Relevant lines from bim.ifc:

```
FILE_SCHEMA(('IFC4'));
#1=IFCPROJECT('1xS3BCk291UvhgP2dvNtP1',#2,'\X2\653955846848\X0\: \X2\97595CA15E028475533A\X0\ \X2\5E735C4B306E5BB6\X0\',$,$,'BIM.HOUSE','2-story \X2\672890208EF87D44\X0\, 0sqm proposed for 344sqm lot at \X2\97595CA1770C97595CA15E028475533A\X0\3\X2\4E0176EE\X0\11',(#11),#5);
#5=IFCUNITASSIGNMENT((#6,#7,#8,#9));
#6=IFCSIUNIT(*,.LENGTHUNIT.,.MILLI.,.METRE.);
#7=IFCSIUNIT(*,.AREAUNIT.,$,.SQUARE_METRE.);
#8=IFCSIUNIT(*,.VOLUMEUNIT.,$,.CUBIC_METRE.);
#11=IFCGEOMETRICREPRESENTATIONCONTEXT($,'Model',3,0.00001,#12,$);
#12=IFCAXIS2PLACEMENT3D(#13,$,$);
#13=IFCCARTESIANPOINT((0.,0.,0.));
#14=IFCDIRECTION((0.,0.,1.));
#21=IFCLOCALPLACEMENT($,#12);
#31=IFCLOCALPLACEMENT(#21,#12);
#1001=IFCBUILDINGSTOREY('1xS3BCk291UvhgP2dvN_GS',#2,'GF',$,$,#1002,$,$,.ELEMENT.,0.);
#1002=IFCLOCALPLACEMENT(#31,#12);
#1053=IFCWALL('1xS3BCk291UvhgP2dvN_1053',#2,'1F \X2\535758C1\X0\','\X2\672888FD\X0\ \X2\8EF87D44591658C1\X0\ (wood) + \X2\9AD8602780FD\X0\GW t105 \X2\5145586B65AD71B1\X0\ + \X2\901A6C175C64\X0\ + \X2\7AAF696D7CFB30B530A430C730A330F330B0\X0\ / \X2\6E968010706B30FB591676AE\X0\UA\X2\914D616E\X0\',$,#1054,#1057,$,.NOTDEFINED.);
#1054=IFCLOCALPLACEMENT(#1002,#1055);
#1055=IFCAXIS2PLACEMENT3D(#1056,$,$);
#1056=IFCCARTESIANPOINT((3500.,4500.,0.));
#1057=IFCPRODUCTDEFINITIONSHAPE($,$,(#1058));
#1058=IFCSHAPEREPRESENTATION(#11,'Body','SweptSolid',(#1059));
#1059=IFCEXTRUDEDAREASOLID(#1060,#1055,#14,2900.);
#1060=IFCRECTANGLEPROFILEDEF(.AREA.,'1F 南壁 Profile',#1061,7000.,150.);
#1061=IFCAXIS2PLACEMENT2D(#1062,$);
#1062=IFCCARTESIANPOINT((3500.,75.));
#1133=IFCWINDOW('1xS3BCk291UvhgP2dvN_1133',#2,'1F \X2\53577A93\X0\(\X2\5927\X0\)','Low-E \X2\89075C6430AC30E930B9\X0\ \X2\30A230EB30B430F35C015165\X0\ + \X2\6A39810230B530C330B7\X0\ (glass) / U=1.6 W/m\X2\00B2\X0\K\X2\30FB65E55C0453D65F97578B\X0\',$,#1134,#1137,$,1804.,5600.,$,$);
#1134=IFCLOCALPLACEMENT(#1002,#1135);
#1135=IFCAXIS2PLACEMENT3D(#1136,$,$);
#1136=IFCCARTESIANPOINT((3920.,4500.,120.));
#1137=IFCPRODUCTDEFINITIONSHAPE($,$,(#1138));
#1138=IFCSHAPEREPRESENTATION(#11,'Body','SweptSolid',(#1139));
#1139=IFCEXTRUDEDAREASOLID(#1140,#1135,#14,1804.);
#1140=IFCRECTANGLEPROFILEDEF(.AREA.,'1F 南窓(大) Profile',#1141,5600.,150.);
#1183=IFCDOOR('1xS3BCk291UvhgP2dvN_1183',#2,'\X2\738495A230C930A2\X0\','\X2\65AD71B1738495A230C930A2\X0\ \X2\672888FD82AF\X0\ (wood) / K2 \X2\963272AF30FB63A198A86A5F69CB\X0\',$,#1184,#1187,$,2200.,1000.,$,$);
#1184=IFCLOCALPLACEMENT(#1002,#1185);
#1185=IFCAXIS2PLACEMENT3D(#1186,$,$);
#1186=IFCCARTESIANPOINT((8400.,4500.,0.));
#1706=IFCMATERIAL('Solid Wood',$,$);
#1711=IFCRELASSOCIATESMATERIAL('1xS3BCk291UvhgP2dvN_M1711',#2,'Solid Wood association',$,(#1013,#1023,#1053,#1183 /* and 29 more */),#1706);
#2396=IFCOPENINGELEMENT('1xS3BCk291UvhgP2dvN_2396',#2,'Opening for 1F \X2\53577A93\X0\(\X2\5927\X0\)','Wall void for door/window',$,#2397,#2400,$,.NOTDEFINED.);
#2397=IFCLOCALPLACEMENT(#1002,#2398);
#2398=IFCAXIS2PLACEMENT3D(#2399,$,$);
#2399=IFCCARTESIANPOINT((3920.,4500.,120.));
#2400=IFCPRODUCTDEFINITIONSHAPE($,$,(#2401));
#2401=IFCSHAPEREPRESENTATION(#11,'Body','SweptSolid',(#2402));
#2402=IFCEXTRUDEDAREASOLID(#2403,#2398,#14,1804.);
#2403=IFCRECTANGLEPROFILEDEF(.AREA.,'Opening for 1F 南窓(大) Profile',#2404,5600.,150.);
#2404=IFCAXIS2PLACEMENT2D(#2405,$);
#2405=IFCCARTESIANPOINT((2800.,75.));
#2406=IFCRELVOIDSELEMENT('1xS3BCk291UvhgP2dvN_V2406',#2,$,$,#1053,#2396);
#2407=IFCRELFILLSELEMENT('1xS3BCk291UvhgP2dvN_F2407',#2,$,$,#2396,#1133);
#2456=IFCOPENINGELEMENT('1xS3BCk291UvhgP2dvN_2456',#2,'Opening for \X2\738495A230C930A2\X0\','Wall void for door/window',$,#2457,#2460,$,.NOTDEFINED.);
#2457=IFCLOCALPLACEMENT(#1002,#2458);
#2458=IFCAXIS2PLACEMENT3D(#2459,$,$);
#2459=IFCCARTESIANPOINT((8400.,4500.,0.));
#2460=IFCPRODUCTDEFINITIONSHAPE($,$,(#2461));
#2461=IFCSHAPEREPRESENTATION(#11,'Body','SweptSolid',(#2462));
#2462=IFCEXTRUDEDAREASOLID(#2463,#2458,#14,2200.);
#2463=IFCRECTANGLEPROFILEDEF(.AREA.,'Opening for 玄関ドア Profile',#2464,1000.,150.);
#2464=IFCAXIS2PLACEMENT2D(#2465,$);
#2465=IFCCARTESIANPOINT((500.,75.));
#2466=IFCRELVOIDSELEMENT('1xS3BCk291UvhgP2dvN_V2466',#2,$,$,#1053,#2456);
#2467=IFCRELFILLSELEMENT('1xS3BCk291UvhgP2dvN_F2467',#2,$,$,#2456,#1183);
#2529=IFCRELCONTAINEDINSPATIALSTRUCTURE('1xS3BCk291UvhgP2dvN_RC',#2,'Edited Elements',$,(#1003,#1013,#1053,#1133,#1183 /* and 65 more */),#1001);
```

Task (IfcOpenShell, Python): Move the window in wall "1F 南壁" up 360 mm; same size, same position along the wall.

```python
import numpy as np
import ifcopenshell
import ifcopenshell.api.geometry
import ifcopenshell.util.placement
import ifcopenshell.util.unit

model = ifcopenshell.open("bim.ifc")
unit_scale = ifcopenshell.util.unit.calculate_unit_scale(model)

window = model.by_guid("1xS3BCk291UvhgP2dvN_1133")
opening = window.FillsVoids[0].RelatingOpeningElement
dz = 0.36 / unit_scale

shift = np.array([0.0, 0.0, dz])
# The window is not placed relative to its opening, so move both.
for product in (opening, window):
    matrix = ifcopenshell.util.placement.get_local_placement(product.ObjectPlacement)
    matrix[:3, 3] += shift
    ifcopenshell.api.geometry.edit_object_placement(model, product=product, matrix=matrix, is_si=False)

print(f"moved by {dz * unit_scale:+.3f} m")

model.write("bim_rev.ifc")
```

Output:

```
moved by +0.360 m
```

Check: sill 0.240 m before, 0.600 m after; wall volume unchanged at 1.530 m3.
